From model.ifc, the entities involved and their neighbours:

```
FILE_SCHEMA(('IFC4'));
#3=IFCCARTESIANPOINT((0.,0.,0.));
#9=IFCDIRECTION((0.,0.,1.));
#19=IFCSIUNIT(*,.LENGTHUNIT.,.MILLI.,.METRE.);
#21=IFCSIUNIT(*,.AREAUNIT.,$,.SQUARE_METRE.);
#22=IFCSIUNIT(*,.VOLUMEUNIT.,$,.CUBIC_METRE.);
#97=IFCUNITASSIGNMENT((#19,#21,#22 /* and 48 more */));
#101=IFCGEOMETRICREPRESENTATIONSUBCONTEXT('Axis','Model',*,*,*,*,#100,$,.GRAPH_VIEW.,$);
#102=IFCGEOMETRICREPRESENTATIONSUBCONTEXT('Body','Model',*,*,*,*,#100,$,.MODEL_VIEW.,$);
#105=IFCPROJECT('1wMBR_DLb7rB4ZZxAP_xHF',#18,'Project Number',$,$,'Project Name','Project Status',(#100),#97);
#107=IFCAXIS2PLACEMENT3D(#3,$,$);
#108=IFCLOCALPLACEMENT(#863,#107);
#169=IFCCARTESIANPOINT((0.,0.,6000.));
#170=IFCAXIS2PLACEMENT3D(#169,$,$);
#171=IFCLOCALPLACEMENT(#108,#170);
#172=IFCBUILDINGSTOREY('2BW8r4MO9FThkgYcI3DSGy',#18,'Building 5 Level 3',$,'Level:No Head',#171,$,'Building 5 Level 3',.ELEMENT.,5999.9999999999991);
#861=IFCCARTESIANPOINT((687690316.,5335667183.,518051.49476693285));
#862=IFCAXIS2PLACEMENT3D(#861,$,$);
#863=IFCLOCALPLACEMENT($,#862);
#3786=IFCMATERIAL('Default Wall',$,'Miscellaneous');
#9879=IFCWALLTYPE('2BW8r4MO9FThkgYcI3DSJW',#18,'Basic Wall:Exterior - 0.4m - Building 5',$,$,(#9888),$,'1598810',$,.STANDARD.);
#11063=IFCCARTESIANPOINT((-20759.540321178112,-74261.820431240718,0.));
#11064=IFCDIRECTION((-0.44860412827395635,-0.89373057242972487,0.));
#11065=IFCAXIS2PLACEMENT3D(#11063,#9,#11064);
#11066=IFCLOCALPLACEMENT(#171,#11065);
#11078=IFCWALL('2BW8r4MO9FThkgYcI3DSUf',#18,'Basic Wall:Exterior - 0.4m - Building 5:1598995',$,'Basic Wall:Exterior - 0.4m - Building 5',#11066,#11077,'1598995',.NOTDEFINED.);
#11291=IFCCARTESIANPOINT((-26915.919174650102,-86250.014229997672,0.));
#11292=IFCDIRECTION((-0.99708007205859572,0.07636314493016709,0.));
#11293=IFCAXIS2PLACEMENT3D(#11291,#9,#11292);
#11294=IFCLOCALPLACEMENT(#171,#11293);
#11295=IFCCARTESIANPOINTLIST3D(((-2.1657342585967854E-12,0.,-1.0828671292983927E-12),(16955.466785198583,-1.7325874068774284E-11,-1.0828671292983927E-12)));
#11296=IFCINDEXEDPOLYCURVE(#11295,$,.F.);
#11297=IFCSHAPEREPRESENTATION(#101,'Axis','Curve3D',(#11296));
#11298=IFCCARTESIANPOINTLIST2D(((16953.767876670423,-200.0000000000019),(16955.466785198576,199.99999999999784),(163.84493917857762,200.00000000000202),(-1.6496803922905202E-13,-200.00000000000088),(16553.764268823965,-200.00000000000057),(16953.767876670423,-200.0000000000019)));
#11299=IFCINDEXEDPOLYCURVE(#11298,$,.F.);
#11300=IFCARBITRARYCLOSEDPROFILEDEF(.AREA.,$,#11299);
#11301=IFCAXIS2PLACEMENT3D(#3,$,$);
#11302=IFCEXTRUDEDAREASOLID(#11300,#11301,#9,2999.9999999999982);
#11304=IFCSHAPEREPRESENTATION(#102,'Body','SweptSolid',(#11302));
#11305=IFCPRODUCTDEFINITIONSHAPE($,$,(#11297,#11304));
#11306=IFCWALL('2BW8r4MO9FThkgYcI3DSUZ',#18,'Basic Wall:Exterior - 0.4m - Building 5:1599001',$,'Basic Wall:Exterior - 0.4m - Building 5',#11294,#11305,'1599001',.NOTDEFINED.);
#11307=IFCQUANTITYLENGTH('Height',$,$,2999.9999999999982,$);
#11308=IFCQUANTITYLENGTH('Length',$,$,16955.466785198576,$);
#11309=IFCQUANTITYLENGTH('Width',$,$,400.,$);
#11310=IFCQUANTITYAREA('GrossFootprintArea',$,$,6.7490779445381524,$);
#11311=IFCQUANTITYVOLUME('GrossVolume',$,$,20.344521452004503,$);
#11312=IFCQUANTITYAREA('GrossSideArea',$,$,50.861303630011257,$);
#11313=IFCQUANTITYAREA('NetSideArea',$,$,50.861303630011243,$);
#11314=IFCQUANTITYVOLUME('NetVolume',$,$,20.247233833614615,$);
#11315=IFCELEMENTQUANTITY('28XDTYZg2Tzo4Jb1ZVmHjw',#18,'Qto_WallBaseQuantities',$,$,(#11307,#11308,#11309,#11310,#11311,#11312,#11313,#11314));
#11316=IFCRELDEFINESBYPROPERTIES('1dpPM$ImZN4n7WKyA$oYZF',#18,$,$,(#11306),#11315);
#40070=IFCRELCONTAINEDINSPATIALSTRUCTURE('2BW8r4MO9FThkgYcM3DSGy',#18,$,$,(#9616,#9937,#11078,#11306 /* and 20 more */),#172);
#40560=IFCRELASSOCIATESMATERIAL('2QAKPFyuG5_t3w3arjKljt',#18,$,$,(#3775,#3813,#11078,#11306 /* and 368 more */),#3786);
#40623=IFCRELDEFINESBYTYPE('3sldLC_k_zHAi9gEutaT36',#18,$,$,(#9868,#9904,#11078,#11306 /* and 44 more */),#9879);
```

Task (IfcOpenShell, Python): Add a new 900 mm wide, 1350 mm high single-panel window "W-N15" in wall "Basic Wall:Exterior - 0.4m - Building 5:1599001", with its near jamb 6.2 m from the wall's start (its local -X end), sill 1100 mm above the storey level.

```python
import numpy as np
import ifcopenshell
import ifcopenshell.api.feature
import ifcopenshell.api.geometry
import ifcopenshell.api.pset
import ifcopenshell.api.root
import ifcopenshell.api.spatial
import ifcopenshell.geom
import ifcopenshell.util.element
import ifcopenshell.util.placement
import ifcopenshell.util.representation
import ifcopenshell.util.shape
import ifcopenshell.util.unit

model = ifcopenshell.open("model.ifc")
unit_scale = ifcopenshell.util.unit.calculate_unit_scale(model)
area_scale = ifcopenshell.util.unit.calculate_unit_scale(model, "AREAUNIT")
volume_scale = ifcopenshell.util.unit.calculate_unit_scale(model, "VOLUMEUNIT")
settings = ifcopenshell.geom.settings()


def volume(element):
    """Net volume in cubic metres, openings subtracted."""
    shape = ifcopenshell.geom.create_shape(settings, element)
    return ifcopenshell.util.shape.get_volume(shape.geometry)


wall = model.by_guid("2BW8r4MO9FThkgYcI3DSUZ")
storey = ifcopenshell.util.element.get_container(wall, ifc_class="IfcBuildingStorey")
context = ifcopenshell.util.representation.get_context(model, "Model", "Body", "MODEL_VIEW")
before = volume(wall)

width, height, from_end, sill = 0.9, 1.35, 6.2, 1.1  # metres

# The wall runs along its own X axis, and the end named is its -X end.
wall_shape = ifcopenshell.geom.create_shape(settings, wall)
x, y, z = ifcopenshell.util.shape.get_vertices(wall_shape.geometry).T
start = x.min() + from_end
face, thickness = float(y.min()), float(y.max() - y.min())
wall_matrix = ifcopenshell.util.placement.get_local_placement(wall.ObjectPlacement)
level = ifcopenshell.util.placement.get_local_placement(storey.ObjectPlacement)[2, 3]


def in_wall(x, y):
    """Placement at x, y metres in the wall's axes, at sill height."""
    matrix = wall_matrix.copy()
    matrix[:, 3] = wall_matrix @ np.array([x / unit_scale, y / unit_scale, 0.0, 1.0])
    matrix[2, 3] = level + sill / unit_scale
    return matrix


# Opening: a box that overshoots both wall faces by 50 mm.
opening = ifcopenshell.api.root.create_entity(model, ifc_class="IfcOpeningElement", predefined_type="OPENING")
box = ifcopenshell.api.geometry.add_wall_representation(
    model, context=context, length=width, height=height, thickness=thickness + 0.1
)
ifcopenshell.api.geometry.assign_representation(model, product=opening, representation=box)
ifcopenshell.api.geometry.edit_object_placement(model, product=opening, matrix=in_wall(start, face - 0.05), is_si=False)
ifcopenshell.api.feature.add_feature(model, feature=opening, element=wall)

window = ifcopenshell.api.root.create_entity(model, ifc_class="IfcWindow", name="W-N15", predefined_type="WINDOW")
window.OverallWidth, window.OverallHeight = width / unit_scale, height / unit_scale
window.PartitioningType = "SINGLE_PANEL"
body = ifcopenshell.api.geometry.add_window_representation(
    model,
    context=context,
    overall_width=window.OverallWidth,
    overall_height=window.OverallHeight,
    partition_type="SINGLE_PANEL",
)
ifcopenshell.api.geometry.assign_representation(model, product=window, representation=body)
ifcopenshell.api.spatial.assign_container(model, products=[window], relating_structure=storey)
ifcopenshell.api.feature.add_filling(model, opening=opening, element=window)

# Centre the window in the wall's thickness.
ifcopenshell.api.geometry.edit_object_placement(model, product=window, matrix=in_wall(start, face), is_si=False)
window_shape = ifcopenshell.geom.create_shape(settings, window)
depth = ifcopenshell.util.shape.get_vertices(window_shape.geometry)[:, 1]
offset = face + thickness / 2 - (depth.min() + depth.max()) / 2
ifcopenshell.api.geometry.edit_object_placement(model, product=window, matrix=in_wall(start, offset), is_si=False)

after = volume(wall)

# Update the wall's stored quantities.
qto = model.by_id(ifcopenshell.util.element.get_pset(wall, "Qto_WallBaseQuantities", should_inherit=False)["id"])
ifcopenshell.api.pset.edit_qto(model, qto=qto, properties={
    "NetSideArea": after / thickness / area_scale,
    "NetVolume": after / volume_scale,
})

print(f"wall volume {before:.3f} -> {after:.3f} m3")

model.write("model_updated.ifc")
```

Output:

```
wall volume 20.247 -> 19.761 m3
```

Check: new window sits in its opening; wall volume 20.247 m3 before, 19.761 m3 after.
